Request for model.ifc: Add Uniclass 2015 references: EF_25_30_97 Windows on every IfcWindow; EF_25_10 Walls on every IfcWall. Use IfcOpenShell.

First a look at what the model holds.

```python
import ifcopenshell

model = ifcopenshell.open("model.ifc")
print(model.schema)
print("classifications:", [c.Name for c in model.by_type("IfcClassification")])
for ifc_class in ("IfcDoor", "IfcRoof", "IfcStair", "IfcWall", "IfcWindow"):
    print(ifc_class, len(model.by_type(ifc_class)))
```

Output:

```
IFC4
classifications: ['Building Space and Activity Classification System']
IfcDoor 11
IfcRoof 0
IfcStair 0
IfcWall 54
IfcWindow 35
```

```python
import ifcopenshell
import ifcopenshell.api.classification

model = ifcopenshell.open("model.ifc")

system = ifcopenshell.api.classification.add_classification(model, classification="Uniclass 2015")

codes = {
    "IfcWindow": ("EF_25_30_97", "Windows"),
    "IfcWall": ("EF_25_10", "Walls"),
}
for ifc_class, (code, name) in codes.items():
    products = model.by_type(ifc_class)
    ifcopenshell.api.classification.add_reference(
        model, products=products, classification=system, identification=code, name=name
    )
    print(code, len(products))

model.write("model_updated.ifc")
```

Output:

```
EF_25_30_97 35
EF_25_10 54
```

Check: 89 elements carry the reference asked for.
